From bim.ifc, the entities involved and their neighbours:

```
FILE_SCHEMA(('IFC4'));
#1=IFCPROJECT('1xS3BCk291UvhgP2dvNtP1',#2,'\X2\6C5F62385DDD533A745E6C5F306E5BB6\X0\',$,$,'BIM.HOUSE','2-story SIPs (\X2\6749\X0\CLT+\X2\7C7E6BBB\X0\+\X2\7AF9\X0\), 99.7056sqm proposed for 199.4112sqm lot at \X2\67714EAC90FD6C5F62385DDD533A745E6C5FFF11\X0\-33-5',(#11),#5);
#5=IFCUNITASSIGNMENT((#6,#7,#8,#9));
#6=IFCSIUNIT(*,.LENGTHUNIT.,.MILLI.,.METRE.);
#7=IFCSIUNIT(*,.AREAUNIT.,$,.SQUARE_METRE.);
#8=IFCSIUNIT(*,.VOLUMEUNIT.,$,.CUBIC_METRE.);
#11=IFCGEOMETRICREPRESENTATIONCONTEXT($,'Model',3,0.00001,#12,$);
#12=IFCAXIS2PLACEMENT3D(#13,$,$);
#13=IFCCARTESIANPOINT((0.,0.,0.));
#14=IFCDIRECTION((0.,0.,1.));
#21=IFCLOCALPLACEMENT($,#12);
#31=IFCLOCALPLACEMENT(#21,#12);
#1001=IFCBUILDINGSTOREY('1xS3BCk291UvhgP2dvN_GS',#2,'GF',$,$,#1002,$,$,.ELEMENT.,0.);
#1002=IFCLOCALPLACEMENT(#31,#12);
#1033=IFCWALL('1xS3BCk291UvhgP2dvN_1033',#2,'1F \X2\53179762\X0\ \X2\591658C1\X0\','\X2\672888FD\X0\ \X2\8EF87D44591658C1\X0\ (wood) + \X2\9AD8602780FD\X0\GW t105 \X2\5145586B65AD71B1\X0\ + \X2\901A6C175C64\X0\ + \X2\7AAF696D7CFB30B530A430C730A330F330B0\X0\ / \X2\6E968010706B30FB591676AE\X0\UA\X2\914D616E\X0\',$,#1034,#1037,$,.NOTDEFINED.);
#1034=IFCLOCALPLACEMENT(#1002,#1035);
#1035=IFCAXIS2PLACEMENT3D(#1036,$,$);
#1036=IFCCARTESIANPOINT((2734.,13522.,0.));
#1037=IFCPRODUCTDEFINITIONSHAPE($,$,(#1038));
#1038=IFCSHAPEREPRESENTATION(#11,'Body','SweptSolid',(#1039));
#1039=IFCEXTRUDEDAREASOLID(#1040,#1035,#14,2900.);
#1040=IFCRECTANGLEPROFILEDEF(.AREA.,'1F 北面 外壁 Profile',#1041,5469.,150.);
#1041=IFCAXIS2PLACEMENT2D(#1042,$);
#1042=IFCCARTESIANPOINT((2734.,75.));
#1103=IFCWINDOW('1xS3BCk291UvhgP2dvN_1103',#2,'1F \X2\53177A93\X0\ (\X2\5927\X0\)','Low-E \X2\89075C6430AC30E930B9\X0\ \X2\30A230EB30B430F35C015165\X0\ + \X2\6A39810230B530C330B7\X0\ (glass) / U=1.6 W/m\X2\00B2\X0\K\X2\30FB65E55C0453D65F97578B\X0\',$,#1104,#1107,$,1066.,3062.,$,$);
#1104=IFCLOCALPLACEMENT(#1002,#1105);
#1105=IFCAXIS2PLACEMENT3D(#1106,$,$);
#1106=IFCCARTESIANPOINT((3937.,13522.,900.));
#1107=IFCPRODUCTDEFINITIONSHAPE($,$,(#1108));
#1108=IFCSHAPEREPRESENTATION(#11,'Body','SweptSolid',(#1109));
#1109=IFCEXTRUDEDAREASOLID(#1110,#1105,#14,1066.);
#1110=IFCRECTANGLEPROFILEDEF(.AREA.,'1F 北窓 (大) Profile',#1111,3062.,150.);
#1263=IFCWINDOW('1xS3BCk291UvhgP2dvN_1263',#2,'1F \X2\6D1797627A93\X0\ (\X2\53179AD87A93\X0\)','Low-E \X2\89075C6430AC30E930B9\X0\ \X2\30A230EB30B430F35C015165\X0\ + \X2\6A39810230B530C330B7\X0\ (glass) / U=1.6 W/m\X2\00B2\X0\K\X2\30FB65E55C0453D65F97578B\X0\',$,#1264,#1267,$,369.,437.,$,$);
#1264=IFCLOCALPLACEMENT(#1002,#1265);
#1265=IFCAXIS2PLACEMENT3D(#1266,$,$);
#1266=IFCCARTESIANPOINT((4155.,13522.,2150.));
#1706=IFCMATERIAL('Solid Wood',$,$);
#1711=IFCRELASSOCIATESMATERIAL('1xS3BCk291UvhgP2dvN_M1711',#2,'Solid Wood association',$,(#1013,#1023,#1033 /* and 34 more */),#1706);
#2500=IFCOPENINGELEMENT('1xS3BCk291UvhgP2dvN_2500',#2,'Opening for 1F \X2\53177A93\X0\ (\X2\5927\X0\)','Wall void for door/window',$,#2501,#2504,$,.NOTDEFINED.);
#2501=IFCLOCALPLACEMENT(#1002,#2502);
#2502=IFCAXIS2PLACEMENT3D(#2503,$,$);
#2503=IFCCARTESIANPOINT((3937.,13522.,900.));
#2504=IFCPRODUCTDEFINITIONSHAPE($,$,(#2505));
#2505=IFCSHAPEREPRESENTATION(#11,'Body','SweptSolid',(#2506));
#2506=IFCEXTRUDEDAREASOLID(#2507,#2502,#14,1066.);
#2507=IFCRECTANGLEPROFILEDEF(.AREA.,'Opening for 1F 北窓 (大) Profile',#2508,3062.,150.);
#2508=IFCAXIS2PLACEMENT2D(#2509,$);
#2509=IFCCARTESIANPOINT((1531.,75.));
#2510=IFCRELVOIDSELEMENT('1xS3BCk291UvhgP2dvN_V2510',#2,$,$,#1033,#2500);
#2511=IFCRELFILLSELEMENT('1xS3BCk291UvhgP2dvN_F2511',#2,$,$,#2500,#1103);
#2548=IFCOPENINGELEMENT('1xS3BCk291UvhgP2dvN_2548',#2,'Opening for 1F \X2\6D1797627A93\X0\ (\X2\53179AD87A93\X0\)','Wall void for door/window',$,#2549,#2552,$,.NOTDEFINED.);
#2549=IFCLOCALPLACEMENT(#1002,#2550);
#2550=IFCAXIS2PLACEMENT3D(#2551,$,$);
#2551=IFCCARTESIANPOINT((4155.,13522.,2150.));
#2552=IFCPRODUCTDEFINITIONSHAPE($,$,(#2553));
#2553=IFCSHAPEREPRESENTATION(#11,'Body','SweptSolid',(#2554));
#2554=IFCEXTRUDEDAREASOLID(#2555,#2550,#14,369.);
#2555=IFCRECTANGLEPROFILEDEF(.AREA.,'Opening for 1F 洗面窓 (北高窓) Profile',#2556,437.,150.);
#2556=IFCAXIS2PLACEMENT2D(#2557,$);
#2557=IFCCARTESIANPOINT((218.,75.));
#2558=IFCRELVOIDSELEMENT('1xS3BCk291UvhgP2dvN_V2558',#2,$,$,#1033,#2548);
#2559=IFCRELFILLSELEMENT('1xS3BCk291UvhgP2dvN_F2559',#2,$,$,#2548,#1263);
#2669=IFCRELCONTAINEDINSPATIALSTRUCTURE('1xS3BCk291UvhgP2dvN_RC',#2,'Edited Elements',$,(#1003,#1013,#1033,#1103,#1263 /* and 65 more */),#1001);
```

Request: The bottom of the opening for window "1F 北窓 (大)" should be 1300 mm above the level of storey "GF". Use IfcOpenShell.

```python
import numpy as np
import ifcopenshell
import ifcopenshell.api.geometry
import ifcopenshell.geom
import ifcopenshell.util.element
import ifcopenshell.util.placement
import ifcopenshell.util.shape
import ifcopenshell.util.unit

model = ifcopenshell.open("bim.ifc")
unit_scale = ifcopenshell.util.unit.calculate_unit_scale(model)

window = model.by_guid("1xS3BCk291UvhgP2dvN_1103")
opening = window.FillsVoids[0].RelatingOpeningElement
storey = ifcopenshell.util.element.get_container(window, ifc_class="IfcBuildingStorey")
level = ifcopenshell.util.placement.get_local_placement(storey.ObjectPlacement)[2, 3]

# The opening's origin need not be at the sill, so measure its lowest point.
shape = ifcopenshell.geom.create_shape(ifcopenshell.geom.settings(), opening)
bottom = ifcopenshell.util.shape.get_shape_bottom_elevation(shape, shape.geometry) / unit_scale
dz = level + 1300.0 - bottom

shift = np.array([0.0, 0.0, dz])
# The window is not placed relative to its opening, so move both.
for product in (opening, window):
    matrix = ifcopenshell.util.placement.get_local_placement(product.ObjectPlacement)
    matrix[:3, 3] += shift
    ifcopenshell.api.geometry.edit_object_placement(model, product=product, matrix=matrix, is_si=False)

print(f"moved by {dz * unit_scale:+.3f} m")

model.write("bim-out.ifc")
```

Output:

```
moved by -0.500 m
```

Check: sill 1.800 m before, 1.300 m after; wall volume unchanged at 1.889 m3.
